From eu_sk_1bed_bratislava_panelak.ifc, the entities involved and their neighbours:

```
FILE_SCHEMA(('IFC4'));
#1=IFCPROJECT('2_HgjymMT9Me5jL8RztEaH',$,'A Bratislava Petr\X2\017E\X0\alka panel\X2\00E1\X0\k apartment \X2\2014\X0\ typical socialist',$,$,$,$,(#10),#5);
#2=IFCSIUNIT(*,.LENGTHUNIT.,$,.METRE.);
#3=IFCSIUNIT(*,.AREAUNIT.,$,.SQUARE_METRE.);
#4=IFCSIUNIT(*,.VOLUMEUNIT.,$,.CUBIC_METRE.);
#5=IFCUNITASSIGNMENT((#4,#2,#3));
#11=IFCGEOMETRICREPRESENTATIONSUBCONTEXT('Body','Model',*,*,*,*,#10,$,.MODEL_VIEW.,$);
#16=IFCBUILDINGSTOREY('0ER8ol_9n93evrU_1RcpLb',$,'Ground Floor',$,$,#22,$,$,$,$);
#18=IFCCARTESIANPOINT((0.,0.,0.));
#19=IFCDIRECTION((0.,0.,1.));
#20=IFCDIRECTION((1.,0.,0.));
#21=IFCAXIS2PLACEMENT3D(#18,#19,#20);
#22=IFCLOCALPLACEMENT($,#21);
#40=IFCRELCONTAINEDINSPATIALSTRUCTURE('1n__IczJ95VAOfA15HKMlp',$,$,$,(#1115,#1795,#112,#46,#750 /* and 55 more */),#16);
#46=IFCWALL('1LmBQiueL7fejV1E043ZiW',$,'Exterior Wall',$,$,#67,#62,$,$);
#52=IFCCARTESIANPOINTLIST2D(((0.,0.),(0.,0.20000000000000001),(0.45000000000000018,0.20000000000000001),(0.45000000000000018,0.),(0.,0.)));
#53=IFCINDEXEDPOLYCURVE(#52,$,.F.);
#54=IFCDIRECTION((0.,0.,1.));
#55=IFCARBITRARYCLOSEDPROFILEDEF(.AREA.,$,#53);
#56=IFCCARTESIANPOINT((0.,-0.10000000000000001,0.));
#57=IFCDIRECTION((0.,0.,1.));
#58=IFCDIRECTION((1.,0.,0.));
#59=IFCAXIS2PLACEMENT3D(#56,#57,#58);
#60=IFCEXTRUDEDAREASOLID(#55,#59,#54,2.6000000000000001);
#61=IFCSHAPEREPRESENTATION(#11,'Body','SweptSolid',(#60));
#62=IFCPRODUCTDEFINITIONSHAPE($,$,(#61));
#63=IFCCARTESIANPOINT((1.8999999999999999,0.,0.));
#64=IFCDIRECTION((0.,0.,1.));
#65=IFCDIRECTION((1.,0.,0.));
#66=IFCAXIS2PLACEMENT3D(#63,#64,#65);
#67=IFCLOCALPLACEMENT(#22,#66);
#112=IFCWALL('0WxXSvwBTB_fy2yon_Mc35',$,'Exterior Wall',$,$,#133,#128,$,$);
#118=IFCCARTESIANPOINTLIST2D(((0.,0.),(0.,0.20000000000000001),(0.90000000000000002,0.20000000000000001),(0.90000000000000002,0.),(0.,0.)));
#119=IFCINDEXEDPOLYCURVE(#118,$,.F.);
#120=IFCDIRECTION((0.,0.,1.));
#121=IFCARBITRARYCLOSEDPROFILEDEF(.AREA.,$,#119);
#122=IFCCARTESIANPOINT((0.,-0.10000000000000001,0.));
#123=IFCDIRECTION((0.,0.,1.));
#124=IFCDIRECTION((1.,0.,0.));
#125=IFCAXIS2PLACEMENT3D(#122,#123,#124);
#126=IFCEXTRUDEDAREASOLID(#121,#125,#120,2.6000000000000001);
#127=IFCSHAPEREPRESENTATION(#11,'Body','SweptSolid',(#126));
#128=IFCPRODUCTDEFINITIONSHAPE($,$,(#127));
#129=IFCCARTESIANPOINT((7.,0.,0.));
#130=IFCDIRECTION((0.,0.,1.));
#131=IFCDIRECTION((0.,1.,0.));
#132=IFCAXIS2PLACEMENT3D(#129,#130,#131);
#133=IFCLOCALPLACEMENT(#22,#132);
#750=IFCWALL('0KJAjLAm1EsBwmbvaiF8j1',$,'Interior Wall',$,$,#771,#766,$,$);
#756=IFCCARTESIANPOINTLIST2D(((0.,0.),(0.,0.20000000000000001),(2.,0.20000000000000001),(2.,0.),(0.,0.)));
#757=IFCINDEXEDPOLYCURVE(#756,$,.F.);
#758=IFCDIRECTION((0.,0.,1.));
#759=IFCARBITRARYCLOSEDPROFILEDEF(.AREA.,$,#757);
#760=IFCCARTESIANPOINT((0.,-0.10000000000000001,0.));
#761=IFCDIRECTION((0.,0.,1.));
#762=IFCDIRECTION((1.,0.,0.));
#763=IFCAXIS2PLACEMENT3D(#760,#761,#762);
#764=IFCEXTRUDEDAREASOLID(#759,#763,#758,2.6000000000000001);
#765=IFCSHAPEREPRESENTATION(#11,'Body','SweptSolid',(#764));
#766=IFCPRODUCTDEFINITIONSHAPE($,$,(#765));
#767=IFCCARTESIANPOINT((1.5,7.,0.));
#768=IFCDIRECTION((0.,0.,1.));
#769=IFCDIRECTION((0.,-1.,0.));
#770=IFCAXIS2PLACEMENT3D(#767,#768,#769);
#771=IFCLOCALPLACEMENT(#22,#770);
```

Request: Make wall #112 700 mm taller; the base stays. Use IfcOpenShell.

```python
import ifcopenshell
import ifcopenshell.geom
import ifcopenshell.util.representation
import ifcopenshell.util.shape
import ifcopenshell.util.unit

model = ifcopenshell.open("eu_sk_1bed_bratislava_panelak.ifc")
unit_scale = ifcopenshell.util.unit.calculate_unit_scale(model)
settings = ifcopenshell.geom.settings()


def volume(element):
    """Net volume in cubic metres, openings subtracted."""
    shape = ifcopenshell.geom.create_shape(settings, element)
    return ifcopenshell.util.shape.get_volume(shape.geometry)


wall = model.by_id(112)
before = volume(wall)

body = ifcopenshell.util.representation.get_representation(wall, "Model", "Body")
solid = body.Items[0]
old_height = solid.Depth
solid.Depth += 0.7 / unit_scale
after = volume(wall)

print(f"height {old_height:g} -> {solid.Depth:g}, volume {before:.3f} -> {after:.3f} m3")

model.write("eu_sk_1bed_bratislava_panelak_v2.ifc")
```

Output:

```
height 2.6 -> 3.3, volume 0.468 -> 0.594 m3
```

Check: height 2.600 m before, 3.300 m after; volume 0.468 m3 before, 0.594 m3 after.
